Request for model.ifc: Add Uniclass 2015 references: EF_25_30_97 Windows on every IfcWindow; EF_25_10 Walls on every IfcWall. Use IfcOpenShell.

First a look at what the model holds.

```python
import ifcopenshell

model = ifcopenshell.open("model.ifc")
print(model.schema)
print("classifications:", [c.Name for c in model.by_type("IfcClassification")])
for ifc_class in ("IfcDoor", "IfcRoof", "IfcStair", "IfcWall", "IfcWindow"):
    print(ifc_class, len(model.by_type(ifc_class)))
```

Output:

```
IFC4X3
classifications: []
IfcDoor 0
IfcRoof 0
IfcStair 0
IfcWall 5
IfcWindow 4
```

```python
import ifcopenshell
import ifcopenshell.api.classification

model = ifcopenshell.open("model.ifc")

system = ifcopenshell.api.classification.add_classification(model, classification="Uniclass 2015")

codes = {
    "IfcWindow": ("EF_25_30_97", "Windows"),
    "IfcWall": ("EF_25_10", "Walls"),
}
for ifc_class, (code, name) in codes.items():
    products = model.by_type(ifc_class)
    ifcopenshell.api.classification.add_reference(
        model, products=products, classification=system, identification=code, name=name
    )
    print(code, len(products))

model.write("model-out.ifc")
```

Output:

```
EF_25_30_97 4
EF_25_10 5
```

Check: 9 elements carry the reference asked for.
